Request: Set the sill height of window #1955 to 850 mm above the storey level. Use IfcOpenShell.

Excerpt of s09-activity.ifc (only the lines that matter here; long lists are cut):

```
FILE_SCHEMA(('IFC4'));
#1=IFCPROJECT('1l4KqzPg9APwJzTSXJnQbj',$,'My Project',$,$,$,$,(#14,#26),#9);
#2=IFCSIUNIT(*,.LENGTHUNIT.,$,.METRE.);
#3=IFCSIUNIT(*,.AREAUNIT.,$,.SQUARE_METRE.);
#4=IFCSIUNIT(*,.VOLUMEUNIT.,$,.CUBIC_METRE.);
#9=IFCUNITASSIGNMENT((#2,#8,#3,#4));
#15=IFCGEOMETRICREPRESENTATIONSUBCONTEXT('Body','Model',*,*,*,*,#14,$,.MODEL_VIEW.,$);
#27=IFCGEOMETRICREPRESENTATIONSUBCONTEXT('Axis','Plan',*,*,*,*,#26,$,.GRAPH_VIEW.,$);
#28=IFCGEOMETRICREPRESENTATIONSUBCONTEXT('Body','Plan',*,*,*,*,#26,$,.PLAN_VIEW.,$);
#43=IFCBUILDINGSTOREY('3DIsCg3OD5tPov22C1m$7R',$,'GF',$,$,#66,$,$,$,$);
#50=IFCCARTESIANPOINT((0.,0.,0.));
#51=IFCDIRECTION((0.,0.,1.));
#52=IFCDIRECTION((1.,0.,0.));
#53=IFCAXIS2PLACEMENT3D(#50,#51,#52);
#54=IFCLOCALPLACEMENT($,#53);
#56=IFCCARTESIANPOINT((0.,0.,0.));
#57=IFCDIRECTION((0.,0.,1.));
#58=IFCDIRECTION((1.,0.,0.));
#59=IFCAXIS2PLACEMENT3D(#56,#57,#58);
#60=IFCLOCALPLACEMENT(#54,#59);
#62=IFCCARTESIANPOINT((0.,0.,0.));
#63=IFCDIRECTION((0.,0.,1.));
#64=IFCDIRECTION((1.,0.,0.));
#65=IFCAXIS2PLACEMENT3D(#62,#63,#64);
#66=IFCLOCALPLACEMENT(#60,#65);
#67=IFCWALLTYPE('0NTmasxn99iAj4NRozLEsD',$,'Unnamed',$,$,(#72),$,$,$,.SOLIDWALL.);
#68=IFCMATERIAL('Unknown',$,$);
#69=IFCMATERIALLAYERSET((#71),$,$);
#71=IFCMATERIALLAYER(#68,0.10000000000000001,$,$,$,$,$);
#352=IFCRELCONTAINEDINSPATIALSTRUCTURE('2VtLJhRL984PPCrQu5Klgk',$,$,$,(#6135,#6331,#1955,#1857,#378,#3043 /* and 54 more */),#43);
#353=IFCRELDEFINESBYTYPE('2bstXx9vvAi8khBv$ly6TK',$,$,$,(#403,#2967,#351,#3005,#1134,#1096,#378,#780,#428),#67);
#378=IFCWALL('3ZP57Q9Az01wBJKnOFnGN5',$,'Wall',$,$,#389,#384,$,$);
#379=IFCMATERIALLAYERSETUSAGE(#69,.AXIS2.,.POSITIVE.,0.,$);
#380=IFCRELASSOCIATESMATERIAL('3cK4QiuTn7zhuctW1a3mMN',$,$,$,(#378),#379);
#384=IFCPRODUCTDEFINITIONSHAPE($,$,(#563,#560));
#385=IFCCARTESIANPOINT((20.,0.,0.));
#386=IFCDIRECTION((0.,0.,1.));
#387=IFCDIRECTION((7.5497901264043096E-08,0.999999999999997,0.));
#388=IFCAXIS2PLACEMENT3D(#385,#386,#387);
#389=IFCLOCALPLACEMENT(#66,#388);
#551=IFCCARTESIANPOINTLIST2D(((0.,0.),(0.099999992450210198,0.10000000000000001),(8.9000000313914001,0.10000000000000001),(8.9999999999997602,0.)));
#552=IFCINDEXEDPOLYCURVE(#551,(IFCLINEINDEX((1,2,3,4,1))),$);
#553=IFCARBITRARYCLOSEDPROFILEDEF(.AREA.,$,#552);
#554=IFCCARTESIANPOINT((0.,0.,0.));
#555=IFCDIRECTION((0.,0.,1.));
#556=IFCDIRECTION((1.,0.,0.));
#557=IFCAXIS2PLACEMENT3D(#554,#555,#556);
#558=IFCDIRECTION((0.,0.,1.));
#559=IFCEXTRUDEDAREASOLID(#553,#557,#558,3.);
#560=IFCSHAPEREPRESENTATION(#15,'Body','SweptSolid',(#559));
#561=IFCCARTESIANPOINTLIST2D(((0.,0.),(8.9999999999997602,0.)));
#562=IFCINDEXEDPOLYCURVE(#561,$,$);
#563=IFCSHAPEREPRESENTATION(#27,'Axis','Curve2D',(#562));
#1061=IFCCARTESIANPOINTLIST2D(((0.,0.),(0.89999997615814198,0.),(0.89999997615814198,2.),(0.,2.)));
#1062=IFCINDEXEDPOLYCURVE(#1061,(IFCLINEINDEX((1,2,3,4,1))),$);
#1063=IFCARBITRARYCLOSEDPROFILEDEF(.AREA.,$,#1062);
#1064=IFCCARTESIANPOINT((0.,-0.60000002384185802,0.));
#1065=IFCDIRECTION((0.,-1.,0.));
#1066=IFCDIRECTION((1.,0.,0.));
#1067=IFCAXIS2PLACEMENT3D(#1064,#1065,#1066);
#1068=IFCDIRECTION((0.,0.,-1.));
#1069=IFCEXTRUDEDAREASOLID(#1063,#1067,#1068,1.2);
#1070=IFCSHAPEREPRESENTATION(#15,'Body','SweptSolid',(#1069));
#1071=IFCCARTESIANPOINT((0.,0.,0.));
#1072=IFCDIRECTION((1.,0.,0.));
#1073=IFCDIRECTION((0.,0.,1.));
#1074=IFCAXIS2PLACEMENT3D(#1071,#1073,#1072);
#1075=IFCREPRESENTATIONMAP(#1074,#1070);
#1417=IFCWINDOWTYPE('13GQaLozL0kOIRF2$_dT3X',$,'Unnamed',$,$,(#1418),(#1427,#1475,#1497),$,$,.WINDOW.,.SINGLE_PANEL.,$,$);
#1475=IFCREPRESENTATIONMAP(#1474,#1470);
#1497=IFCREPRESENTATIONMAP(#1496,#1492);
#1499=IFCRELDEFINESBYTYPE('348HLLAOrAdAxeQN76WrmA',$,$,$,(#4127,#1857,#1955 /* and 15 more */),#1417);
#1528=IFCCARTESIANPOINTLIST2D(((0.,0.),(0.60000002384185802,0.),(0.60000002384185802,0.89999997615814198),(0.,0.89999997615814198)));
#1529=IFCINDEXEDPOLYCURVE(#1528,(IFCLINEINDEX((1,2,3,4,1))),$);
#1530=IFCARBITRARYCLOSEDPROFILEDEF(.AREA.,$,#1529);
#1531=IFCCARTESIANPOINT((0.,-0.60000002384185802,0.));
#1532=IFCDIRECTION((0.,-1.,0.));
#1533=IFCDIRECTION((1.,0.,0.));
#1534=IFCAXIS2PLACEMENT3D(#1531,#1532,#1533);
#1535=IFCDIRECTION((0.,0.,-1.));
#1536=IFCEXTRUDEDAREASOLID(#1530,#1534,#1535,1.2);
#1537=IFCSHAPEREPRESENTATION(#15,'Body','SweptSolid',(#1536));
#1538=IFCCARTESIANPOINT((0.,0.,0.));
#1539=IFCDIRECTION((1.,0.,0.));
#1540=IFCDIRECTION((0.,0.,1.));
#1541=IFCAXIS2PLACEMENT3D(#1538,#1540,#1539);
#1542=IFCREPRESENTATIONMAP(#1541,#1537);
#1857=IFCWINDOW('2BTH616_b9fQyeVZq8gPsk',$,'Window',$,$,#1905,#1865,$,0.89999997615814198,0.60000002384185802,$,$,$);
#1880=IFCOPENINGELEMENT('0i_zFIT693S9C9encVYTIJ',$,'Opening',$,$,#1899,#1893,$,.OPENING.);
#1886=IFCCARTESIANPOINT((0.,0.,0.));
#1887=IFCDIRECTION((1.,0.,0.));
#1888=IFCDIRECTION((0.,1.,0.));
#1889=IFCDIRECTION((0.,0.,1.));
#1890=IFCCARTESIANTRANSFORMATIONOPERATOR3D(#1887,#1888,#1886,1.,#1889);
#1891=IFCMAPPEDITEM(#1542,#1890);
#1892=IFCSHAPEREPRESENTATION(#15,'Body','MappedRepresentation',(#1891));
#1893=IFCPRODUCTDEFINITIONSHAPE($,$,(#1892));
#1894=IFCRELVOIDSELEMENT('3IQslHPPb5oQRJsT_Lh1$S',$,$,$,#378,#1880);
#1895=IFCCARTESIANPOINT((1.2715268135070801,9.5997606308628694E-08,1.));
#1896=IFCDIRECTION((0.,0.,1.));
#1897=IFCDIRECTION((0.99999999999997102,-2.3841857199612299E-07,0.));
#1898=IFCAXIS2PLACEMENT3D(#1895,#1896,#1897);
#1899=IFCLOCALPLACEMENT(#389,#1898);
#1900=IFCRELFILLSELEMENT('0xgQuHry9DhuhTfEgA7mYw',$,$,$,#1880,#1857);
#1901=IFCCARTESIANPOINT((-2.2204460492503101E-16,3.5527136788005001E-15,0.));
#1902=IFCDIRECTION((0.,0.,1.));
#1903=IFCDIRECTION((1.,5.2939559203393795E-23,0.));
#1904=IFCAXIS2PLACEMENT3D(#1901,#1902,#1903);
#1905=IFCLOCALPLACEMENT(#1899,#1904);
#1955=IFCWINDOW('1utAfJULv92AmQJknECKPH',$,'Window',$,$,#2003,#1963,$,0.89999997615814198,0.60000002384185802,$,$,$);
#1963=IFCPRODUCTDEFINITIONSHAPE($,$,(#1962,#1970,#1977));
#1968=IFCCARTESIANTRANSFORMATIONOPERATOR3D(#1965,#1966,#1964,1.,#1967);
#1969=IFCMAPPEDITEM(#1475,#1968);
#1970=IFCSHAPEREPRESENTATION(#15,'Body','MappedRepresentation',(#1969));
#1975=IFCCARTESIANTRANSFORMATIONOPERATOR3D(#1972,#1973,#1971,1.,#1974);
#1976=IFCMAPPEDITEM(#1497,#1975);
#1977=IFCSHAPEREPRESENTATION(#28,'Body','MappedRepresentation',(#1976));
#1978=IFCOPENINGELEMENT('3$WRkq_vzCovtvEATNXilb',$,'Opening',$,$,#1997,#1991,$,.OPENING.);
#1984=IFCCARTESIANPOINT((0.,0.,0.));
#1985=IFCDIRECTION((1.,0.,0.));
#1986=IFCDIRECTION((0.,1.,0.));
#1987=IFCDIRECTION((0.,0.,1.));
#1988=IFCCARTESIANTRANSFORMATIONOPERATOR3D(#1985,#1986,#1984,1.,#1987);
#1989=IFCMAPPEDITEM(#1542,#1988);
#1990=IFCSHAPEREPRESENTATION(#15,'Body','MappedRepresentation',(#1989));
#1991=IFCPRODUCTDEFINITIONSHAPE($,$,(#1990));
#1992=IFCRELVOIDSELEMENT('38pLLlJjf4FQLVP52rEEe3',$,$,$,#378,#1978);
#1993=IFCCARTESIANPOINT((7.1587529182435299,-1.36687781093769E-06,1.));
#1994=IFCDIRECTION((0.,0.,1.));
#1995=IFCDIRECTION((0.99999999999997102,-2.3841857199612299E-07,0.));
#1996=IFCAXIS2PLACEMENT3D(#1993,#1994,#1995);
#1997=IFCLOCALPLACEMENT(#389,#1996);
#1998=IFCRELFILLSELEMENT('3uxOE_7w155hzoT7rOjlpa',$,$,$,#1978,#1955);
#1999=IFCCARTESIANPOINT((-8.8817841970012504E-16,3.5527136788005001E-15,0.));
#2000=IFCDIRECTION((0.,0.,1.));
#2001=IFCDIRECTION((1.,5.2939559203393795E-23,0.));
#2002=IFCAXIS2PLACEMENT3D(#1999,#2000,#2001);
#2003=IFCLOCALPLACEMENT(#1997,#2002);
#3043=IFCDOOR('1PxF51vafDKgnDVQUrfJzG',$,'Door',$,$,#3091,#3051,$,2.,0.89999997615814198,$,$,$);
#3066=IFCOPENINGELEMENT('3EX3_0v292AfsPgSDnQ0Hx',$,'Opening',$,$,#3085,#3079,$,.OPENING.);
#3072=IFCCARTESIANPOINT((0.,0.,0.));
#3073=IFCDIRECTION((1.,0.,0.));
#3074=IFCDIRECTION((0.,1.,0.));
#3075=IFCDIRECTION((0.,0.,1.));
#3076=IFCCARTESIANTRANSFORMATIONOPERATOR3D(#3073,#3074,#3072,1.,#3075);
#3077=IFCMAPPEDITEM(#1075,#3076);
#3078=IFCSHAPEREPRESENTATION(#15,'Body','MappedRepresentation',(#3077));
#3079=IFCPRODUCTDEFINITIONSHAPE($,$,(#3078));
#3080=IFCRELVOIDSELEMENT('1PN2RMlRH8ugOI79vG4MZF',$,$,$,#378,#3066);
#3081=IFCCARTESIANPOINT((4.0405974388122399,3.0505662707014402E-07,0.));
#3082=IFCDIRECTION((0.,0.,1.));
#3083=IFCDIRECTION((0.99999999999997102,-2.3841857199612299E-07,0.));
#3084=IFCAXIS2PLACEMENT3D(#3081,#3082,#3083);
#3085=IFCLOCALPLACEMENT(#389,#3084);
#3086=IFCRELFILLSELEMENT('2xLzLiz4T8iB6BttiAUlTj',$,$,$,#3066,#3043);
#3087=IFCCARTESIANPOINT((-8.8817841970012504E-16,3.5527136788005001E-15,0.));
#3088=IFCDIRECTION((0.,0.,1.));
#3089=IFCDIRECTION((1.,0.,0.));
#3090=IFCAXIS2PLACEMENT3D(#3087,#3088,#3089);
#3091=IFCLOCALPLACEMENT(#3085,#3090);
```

```python
import numpy as np
import ifcopenshell
import ifcopenshell.api.geometry
import ifcopenshell.geom
import ifcopenshell.util.element
import ifcopenshell.util.placement
import ifcopenshell.util.shape
import ifcopenshell.util.unit

model = ifcopenshell.open("s09-activity.ifc")
unit_scale = ifcopenshell.util.unit.calculate_unit_scale(model)

window = model.by_guid("1utAfJULv92AmQJknECKPH")
opening = window.FillsVoids[0].RelatingOpeningElement
storey = ifcopenshell.util.element.get_container(window, ifc_class="IfcBuildingStorey")
level = ifcopenshell.util.placement.get_local_placement(storey.ObjectPlacement)[2, 3]

# The opening's origin need not be at the sill, so measure its lowest point.
shape = ifcopenshell.geom.create_shape(ifcopenshell.geom.settings(), opening)
bottom = ifcopenshell.util.shape.get_shape_bottom_elevation(shape, shape.geometry) / unit_scale
dz = level + 0.85 / unit_scale - bottom

shift = np.array([0.0, 0.0, dz])
# The window is placed relative to its opening, so it follows when the opening moves.
matrix = ifcopenshell.util.placement.get_local_placement(opening.ObjectPlacement)
matrix[:3, 3] += shift
ifcopenshell.api.geometry.edit_object_placement(
    model, product=opening, matrix=matrix, is_si=False, should_transform_children=True
)

print(f"moved by {dz * unit_scale:+.3f} m")

model.write("s09-activity_updated.ifc")
```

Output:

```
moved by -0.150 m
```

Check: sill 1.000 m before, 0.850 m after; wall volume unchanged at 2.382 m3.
